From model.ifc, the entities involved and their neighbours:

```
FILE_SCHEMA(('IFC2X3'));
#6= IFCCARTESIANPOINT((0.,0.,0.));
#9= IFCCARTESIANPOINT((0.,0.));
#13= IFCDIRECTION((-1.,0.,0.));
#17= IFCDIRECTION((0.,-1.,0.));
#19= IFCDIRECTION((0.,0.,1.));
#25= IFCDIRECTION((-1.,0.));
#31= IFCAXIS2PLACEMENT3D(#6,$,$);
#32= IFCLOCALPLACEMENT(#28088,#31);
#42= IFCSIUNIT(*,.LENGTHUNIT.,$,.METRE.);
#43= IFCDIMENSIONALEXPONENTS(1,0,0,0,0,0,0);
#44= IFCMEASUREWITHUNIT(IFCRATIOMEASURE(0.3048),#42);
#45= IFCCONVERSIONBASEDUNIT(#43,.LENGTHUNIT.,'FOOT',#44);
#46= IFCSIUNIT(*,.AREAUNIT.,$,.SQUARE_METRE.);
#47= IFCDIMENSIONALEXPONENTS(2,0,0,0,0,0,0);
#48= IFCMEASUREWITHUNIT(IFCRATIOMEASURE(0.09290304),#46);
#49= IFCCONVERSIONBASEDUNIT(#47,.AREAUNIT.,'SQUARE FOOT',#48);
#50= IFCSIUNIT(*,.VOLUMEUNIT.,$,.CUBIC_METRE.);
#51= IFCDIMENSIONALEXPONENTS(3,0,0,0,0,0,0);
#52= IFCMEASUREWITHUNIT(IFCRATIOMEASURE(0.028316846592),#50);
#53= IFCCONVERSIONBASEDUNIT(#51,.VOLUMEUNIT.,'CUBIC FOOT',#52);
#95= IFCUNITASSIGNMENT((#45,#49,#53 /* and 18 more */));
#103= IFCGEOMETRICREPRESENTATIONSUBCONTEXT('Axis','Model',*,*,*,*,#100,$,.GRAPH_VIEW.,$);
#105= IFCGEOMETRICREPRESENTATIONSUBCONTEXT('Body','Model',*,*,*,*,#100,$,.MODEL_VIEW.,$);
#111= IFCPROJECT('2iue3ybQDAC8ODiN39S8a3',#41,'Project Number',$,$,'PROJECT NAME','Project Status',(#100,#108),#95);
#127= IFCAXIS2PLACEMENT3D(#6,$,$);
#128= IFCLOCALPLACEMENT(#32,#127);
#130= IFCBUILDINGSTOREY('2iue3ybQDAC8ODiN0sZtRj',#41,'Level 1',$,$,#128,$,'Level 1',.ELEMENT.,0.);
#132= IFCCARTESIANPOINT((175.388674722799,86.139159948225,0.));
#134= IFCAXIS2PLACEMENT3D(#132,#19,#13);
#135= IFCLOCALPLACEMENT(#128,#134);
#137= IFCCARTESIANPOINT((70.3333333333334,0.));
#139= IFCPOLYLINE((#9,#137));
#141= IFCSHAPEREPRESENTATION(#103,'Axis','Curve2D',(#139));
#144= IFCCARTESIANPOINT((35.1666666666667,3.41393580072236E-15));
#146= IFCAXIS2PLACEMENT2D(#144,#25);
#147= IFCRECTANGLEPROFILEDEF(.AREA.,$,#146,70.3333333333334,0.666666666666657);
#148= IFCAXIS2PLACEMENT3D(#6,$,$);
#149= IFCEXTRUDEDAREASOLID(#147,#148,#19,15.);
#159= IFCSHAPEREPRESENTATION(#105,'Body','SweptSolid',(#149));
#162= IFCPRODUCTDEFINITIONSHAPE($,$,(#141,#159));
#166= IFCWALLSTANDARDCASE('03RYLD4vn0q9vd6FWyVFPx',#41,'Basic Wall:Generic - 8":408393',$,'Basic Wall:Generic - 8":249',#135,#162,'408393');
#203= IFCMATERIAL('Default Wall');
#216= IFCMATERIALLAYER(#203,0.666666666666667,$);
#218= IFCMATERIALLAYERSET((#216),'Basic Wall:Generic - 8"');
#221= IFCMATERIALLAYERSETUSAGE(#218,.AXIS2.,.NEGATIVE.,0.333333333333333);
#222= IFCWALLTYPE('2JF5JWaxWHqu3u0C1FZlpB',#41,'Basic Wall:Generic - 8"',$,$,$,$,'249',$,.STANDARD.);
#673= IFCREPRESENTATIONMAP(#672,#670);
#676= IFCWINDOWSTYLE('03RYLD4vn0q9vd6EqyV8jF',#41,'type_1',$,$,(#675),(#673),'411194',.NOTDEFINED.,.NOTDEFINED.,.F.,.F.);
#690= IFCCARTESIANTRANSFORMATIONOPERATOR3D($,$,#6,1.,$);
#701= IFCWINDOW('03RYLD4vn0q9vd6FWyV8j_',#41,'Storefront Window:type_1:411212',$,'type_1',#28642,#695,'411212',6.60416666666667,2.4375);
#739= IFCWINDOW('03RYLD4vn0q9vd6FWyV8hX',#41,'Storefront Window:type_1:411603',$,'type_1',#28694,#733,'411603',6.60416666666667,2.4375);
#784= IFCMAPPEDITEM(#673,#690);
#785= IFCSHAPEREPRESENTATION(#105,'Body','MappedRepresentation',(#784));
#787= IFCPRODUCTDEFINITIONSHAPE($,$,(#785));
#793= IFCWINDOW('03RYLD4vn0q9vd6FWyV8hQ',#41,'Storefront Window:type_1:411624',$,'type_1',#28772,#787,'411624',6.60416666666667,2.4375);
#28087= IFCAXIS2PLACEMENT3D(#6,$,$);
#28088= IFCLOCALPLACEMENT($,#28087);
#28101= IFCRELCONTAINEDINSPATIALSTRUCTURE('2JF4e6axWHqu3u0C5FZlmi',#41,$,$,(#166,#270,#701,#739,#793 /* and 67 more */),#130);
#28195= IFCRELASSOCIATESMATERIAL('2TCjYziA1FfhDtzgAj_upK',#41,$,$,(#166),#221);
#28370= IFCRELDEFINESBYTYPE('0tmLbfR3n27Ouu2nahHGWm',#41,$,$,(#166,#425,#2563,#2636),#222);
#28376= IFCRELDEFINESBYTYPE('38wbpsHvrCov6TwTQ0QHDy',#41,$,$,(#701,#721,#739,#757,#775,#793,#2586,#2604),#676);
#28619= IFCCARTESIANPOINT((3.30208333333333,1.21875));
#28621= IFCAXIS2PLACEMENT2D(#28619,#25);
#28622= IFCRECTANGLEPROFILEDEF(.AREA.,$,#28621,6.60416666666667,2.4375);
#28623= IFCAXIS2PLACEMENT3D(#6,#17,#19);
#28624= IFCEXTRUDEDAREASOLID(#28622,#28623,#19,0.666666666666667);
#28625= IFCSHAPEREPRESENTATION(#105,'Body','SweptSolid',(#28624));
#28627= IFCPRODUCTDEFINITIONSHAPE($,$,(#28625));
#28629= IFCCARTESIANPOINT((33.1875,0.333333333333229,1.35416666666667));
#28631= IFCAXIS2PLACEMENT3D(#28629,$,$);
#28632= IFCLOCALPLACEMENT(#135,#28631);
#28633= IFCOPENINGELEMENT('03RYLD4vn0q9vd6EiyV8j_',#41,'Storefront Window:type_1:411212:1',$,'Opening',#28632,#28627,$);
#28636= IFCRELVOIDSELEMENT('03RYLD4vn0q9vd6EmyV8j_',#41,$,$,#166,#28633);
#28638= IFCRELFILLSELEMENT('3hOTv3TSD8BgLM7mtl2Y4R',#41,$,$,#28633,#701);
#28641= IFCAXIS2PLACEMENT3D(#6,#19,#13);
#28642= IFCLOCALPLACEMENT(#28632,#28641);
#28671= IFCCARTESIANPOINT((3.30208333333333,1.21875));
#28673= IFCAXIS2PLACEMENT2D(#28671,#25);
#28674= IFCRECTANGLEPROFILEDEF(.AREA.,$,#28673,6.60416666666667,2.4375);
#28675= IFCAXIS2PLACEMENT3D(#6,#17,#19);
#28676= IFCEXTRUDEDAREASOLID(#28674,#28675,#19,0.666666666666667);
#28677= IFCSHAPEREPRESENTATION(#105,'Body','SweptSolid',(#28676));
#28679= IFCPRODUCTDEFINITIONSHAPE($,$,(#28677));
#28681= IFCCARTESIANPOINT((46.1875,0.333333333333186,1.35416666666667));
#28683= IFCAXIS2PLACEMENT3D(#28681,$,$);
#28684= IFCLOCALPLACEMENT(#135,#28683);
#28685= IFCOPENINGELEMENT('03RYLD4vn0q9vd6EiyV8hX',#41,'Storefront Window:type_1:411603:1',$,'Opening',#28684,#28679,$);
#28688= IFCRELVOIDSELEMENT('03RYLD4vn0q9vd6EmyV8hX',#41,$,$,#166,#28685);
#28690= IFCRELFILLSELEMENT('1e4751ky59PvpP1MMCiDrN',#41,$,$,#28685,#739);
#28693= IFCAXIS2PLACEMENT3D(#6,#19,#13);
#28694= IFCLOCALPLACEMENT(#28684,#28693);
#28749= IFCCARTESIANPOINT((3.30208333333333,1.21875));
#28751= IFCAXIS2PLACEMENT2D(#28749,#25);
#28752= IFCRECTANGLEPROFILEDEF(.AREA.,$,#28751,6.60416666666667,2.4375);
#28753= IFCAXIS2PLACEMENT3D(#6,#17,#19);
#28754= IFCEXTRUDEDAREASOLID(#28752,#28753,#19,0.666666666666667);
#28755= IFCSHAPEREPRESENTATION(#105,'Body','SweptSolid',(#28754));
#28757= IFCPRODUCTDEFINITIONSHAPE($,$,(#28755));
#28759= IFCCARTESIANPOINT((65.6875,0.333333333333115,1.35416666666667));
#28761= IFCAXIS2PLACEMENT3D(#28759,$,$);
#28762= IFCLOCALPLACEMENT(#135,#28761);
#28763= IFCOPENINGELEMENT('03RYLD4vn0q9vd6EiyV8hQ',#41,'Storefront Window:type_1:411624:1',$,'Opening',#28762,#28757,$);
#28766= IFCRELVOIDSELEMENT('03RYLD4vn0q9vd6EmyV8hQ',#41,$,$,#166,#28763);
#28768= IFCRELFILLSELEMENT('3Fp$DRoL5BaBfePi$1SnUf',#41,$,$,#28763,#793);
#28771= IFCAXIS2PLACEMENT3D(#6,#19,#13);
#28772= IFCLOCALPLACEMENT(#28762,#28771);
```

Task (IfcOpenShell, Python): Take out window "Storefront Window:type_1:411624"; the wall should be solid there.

```python
import ifcopenshell
import ifcopenshell.api.feature
import ifcopenshell.api.root
import ifcopenshell.geom
import ifcopenshell.util.shape

model = ifcopenshell.open("model.ifc")
settings = ifcopenshell.geom.settings()


def volume(element):
    """Net volume in cubic metres, openings subtracted."""
    shape = ifcopenshell.geom.create_shape(settings, element)
    return ifcopenshell.util.shape.get_volume(shape.geometry)


window = model.by_guid("03RYLD4vn0q9vd6FWyV8hQ")
opening = window.FillsVoids[0].RelatingOpeningElement
wall = opening.VoidsElements[0].RelatingBuildingElement
before = volume(wall)

ifcopenshell.api.root.remove_product(model, product=window)
ifcopenshell.api.feature.remove_feature(model, feature=opening)

after = volume(wall)

print(f"wall volume {before:.3f} -> {after:.3f} m3")

model.write("model_rev.ifc")
```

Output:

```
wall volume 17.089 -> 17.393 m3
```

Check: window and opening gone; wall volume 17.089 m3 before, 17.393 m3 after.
